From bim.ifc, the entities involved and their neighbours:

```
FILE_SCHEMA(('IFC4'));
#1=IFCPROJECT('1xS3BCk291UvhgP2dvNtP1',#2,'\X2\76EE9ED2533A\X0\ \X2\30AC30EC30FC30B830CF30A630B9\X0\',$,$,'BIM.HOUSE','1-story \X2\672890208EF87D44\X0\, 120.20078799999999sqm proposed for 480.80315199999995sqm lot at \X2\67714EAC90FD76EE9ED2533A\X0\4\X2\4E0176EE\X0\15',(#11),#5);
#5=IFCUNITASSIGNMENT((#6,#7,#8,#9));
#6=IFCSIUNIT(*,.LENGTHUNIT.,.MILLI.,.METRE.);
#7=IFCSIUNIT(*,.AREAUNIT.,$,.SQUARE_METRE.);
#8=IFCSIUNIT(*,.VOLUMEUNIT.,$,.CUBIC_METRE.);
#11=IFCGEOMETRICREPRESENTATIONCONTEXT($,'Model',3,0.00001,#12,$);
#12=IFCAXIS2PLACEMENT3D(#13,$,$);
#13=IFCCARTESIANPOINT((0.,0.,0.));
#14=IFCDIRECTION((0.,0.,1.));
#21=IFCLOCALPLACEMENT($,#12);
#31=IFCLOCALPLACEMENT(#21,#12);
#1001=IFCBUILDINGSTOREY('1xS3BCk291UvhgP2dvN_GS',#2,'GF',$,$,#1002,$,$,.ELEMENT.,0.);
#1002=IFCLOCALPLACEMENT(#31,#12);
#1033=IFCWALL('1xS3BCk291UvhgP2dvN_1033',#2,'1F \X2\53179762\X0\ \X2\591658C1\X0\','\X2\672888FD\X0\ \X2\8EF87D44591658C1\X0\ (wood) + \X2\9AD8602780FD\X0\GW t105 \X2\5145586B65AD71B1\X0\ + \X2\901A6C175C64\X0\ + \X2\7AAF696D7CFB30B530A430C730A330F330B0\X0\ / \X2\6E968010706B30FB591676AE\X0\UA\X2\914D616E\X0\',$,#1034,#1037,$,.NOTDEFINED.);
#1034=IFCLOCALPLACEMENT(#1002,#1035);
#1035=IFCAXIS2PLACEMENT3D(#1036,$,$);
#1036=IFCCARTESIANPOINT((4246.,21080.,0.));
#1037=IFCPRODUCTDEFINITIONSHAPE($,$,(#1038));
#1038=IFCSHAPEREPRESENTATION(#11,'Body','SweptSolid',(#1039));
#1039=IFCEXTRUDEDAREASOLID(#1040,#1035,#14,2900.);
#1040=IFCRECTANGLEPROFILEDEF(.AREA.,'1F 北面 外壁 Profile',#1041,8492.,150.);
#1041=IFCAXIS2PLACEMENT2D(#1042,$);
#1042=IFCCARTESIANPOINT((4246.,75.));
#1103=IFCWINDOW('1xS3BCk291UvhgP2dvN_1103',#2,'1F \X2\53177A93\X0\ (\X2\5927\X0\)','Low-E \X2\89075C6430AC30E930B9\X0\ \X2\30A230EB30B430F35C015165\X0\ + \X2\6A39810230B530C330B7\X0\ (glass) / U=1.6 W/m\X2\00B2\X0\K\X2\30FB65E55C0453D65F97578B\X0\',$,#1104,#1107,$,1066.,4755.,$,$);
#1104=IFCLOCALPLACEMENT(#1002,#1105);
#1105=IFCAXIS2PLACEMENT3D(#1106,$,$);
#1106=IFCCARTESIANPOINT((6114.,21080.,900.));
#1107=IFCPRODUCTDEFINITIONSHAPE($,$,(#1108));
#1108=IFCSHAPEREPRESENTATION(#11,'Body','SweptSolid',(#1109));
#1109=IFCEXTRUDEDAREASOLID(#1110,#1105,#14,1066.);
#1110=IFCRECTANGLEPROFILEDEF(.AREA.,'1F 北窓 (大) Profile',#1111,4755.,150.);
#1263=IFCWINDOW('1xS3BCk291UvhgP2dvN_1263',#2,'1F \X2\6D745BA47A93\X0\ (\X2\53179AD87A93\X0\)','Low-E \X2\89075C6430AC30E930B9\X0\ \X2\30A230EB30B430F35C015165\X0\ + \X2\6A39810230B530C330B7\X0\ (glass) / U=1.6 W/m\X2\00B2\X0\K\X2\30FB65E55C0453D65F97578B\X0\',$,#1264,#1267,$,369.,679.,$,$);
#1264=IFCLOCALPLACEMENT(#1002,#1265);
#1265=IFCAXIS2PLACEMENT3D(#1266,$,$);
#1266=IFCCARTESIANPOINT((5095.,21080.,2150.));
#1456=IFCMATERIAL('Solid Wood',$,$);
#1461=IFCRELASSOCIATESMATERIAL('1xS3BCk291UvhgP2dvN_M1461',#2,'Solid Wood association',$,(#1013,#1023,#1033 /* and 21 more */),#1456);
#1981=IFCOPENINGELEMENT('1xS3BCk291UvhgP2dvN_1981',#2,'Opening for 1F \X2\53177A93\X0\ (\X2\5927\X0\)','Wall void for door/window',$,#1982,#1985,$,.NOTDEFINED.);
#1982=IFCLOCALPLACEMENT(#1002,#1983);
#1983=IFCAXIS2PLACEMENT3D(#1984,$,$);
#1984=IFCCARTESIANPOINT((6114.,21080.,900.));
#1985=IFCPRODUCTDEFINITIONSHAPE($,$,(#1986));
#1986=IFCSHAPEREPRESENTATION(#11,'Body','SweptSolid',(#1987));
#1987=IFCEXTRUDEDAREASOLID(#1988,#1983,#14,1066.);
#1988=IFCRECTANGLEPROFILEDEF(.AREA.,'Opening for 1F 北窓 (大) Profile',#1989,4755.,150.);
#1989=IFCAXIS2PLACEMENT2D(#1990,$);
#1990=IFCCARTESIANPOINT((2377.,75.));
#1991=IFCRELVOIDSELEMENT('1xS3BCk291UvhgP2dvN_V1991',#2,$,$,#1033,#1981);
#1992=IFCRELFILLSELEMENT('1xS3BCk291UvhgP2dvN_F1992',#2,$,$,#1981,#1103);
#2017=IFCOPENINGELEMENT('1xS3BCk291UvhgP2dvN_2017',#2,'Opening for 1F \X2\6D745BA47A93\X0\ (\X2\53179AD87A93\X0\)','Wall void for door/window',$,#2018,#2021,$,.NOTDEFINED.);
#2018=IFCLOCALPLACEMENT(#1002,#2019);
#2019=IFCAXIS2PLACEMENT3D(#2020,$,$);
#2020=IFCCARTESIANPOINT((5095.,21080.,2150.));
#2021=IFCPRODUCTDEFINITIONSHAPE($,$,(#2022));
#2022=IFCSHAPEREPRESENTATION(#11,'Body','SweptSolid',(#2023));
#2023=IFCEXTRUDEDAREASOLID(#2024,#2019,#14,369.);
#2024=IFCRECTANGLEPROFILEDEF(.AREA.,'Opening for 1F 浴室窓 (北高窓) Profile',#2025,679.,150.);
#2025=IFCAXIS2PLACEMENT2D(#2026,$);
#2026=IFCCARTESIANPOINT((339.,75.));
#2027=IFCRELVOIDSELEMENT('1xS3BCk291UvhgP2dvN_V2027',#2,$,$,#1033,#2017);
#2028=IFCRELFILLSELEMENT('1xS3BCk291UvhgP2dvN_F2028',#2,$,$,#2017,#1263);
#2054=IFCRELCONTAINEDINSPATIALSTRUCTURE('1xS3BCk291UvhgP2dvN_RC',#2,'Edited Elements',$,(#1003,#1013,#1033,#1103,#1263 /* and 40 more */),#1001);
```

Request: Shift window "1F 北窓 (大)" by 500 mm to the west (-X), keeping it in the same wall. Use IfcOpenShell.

```python
import ifcopenshell
import ifcopenshell.api.geometry
import ifcopenshell.util.placement
import ifcopenshell.util.unit

model = ifcopenshell.open("bim.ifc")
unit_scale = ifcopenshell.util.unit.calculate_unit_scale(model)

window = model.by_guid("1xS3BCk291UvhgP2dvN_1103")
opening = window.FillsVoids[0].RelatingOpeningElement
wall = opening.VoidsElements[0].RelatingBuildingElement

wall_matrix = ifcopenshell.util.placement.get_local_placement(wall.ObjectPlacement)
shift = wall_matrix[:3, 0] * -0.5 / unit_scale
before = ifcopenshell.util.placement.get_local_placement(window.ObjectPlacement)[:3, 3].copy()

# The window is not placed relative to its opening, so move both.
for product in (opening, window):
    matrix = ifcopenshell.util.placement.get_local_placement(product.ObjectPlacement)
    matrix[:3, 3] += shift
    ifcopenshell.api.geometry.edit_object_placement(model, product=product, matrix=matrix, is_si=False)

after = ifcopenshell.util.placement.get_local_placement(window.ObjectPlacement)[:3, 3]
print("window moved by", (after - before).round(3) + 0.0)

model.write("bim_edited.ifc")
```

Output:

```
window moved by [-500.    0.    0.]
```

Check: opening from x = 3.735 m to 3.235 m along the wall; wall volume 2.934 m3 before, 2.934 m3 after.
